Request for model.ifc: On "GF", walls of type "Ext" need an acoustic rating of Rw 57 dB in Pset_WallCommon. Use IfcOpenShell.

First a look at what the model holds.

```python
import ifcopenshell
import ifcopenshell.util.element

model = ifcopenshell.open("model.ifc")
print(model.schema)
storey = next(s for s in model.by_type("IfcBuildingStorey") if s.Name == "GF")
walls = [e for e in ifcopenshell.util.element.get_decomposition(storey) if e.is_a("IfcWall")]
seen = {}
for e in walls:
    element_type = ifcopenshell.util.element.get_type(e)
    key = (element_type.Name if element_type != e and element_type else None, ifcopenshell.util.element.get_pset(e, "Pset_WallCommon", "AcousticRating"))
    seen[key] = seen.get(key, 0) + 1
for (name, value), count in sorted(seen.items(), key=str):
    print(count, "x", name, "|", value)
```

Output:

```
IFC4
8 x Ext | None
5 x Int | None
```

```python
import ifcopenshell
import ifcopenshell.api.pset
import ifcopenshell.util.element

model = ifcopenshell.open("model.ifc")

storey = next(s for s in model.by_type("IfcBuildingStorey") if s.Name == "GF")
walls = [e for e in ifcopenshell.util.element.get_decomposition(storey) if e.is_a("IfcWall")]

count = 0
for e in walls:
    element_type = ifcopenshell.util.element.get_type(e)
    if element_type in (None, e) or element_type.Name != "Ext":
        continue
    # add_pset returns the element's existing set when there is one.
    pset = ifcopenshell.api.pset.add_pset(model, product=e, name="Pset_WallCommon")
    ifcopenshell.api.pset.edit_pset(model, pset=pset, properties={"AcousticRating": "Rw 57 dB"})
    count += 1

print(count, "walls updated")

model.write("model-out.ifc")
```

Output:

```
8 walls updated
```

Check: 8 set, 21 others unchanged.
